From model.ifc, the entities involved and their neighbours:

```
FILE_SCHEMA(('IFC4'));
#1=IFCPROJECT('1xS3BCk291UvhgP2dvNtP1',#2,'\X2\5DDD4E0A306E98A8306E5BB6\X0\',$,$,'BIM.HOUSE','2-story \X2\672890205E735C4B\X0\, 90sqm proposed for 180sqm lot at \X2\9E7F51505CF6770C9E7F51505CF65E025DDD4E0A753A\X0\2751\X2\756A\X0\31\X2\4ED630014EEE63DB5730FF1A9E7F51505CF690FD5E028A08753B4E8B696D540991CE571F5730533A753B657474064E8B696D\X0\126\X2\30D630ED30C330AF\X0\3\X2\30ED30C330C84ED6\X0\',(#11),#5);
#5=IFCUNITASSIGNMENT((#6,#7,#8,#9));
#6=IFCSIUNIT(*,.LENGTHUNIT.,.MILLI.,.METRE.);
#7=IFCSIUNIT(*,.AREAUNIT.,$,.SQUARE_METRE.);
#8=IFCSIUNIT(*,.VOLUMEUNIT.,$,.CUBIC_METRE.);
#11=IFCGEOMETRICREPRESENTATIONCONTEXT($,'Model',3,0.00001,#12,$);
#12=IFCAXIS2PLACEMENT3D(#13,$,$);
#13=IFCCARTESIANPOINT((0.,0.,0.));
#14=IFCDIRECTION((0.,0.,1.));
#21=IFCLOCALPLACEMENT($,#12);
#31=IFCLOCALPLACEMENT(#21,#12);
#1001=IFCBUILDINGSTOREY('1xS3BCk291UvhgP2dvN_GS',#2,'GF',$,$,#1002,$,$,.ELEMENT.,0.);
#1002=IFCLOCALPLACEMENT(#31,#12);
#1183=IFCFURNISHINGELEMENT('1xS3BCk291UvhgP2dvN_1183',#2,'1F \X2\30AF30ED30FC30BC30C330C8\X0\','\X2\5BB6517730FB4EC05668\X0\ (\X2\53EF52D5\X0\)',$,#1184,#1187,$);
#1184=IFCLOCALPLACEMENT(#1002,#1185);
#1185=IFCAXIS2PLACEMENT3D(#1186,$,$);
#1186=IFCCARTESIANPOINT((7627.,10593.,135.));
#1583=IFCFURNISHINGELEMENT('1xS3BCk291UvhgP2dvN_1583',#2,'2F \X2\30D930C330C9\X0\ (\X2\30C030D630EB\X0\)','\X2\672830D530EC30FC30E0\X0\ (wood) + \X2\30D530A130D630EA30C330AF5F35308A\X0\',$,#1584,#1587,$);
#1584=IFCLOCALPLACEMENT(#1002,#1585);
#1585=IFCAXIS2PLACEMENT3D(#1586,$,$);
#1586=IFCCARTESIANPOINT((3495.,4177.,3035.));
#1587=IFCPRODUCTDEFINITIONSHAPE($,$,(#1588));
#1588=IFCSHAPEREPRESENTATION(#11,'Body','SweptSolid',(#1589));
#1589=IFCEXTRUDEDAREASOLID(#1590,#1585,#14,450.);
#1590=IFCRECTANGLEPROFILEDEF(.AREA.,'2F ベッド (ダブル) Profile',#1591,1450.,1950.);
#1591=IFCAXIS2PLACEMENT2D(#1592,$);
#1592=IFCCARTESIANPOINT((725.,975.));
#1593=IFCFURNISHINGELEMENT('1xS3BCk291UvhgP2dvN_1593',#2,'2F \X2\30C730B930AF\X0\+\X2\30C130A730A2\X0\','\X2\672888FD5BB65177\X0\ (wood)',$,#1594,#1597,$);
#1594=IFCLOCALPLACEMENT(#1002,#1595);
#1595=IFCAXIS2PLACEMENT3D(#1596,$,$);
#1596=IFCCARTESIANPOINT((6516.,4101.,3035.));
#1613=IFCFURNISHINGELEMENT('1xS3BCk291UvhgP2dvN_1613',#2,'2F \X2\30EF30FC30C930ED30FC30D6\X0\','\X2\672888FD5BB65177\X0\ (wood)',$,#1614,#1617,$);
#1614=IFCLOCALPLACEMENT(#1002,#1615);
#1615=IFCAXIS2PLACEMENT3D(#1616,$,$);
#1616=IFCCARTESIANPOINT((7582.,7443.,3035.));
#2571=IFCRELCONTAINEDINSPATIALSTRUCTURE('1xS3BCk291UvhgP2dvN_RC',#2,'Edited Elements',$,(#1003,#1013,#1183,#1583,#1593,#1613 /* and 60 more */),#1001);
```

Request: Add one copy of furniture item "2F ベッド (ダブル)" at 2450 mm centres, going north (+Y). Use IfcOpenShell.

```python
import numpy as np
import ifcopenshell
import ifcopenshell.api.geometry
import ifcopenshell.api.root
import ifcopenshell.util.element
import ifcopenshell.util.placement

model = ifcopenshell.open("model.ifc")


def reuse_history(source, copy):
    """copy_class also copies each property set's owner history, people and application; keep the originals."""
    for rel in copy.IsDefinedBy:
        if rel.is_a("IfcRelDefinesByProperties") and (history := rel.RelatingPropertyDefinition.OwnerHistory):
            rel.RelatingPropertyDefinition.OwnerHistory = source.OwnerHistory
            ifcopenshell.util.element.remove_deep2(model, history)


source = model.by_id(1583)
base = ifcopenshell.util.placement.get_local_placement(source.ObjectPlacement)
step = np.array([0.0, 1.0, 0.0]) * 2450.0

for i in range(1, 2):
    copy = ifcopenshell.api.root.copy_class(model, product=source)
    copy.Representation = ifcopenshell.util.element.copy_deep(
        model, source.Representation, exclude=["IfcGeometricRepresentationContext", "IfcRepresentationMap"]
    )
    reuse_history(source, copy)
    matrix = base.copy()
    matrix[:3, 3] += i * step
    print("added at", matrix[:3, 3].round(3) + 0.0)
    ifcopenshell.api.geometry.edit_object_placement(model, product=copy, matrix=matrix, is_si=False)

model.write("model-out.ifc")
```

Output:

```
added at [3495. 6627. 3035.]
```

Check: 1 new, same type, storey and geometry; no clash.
